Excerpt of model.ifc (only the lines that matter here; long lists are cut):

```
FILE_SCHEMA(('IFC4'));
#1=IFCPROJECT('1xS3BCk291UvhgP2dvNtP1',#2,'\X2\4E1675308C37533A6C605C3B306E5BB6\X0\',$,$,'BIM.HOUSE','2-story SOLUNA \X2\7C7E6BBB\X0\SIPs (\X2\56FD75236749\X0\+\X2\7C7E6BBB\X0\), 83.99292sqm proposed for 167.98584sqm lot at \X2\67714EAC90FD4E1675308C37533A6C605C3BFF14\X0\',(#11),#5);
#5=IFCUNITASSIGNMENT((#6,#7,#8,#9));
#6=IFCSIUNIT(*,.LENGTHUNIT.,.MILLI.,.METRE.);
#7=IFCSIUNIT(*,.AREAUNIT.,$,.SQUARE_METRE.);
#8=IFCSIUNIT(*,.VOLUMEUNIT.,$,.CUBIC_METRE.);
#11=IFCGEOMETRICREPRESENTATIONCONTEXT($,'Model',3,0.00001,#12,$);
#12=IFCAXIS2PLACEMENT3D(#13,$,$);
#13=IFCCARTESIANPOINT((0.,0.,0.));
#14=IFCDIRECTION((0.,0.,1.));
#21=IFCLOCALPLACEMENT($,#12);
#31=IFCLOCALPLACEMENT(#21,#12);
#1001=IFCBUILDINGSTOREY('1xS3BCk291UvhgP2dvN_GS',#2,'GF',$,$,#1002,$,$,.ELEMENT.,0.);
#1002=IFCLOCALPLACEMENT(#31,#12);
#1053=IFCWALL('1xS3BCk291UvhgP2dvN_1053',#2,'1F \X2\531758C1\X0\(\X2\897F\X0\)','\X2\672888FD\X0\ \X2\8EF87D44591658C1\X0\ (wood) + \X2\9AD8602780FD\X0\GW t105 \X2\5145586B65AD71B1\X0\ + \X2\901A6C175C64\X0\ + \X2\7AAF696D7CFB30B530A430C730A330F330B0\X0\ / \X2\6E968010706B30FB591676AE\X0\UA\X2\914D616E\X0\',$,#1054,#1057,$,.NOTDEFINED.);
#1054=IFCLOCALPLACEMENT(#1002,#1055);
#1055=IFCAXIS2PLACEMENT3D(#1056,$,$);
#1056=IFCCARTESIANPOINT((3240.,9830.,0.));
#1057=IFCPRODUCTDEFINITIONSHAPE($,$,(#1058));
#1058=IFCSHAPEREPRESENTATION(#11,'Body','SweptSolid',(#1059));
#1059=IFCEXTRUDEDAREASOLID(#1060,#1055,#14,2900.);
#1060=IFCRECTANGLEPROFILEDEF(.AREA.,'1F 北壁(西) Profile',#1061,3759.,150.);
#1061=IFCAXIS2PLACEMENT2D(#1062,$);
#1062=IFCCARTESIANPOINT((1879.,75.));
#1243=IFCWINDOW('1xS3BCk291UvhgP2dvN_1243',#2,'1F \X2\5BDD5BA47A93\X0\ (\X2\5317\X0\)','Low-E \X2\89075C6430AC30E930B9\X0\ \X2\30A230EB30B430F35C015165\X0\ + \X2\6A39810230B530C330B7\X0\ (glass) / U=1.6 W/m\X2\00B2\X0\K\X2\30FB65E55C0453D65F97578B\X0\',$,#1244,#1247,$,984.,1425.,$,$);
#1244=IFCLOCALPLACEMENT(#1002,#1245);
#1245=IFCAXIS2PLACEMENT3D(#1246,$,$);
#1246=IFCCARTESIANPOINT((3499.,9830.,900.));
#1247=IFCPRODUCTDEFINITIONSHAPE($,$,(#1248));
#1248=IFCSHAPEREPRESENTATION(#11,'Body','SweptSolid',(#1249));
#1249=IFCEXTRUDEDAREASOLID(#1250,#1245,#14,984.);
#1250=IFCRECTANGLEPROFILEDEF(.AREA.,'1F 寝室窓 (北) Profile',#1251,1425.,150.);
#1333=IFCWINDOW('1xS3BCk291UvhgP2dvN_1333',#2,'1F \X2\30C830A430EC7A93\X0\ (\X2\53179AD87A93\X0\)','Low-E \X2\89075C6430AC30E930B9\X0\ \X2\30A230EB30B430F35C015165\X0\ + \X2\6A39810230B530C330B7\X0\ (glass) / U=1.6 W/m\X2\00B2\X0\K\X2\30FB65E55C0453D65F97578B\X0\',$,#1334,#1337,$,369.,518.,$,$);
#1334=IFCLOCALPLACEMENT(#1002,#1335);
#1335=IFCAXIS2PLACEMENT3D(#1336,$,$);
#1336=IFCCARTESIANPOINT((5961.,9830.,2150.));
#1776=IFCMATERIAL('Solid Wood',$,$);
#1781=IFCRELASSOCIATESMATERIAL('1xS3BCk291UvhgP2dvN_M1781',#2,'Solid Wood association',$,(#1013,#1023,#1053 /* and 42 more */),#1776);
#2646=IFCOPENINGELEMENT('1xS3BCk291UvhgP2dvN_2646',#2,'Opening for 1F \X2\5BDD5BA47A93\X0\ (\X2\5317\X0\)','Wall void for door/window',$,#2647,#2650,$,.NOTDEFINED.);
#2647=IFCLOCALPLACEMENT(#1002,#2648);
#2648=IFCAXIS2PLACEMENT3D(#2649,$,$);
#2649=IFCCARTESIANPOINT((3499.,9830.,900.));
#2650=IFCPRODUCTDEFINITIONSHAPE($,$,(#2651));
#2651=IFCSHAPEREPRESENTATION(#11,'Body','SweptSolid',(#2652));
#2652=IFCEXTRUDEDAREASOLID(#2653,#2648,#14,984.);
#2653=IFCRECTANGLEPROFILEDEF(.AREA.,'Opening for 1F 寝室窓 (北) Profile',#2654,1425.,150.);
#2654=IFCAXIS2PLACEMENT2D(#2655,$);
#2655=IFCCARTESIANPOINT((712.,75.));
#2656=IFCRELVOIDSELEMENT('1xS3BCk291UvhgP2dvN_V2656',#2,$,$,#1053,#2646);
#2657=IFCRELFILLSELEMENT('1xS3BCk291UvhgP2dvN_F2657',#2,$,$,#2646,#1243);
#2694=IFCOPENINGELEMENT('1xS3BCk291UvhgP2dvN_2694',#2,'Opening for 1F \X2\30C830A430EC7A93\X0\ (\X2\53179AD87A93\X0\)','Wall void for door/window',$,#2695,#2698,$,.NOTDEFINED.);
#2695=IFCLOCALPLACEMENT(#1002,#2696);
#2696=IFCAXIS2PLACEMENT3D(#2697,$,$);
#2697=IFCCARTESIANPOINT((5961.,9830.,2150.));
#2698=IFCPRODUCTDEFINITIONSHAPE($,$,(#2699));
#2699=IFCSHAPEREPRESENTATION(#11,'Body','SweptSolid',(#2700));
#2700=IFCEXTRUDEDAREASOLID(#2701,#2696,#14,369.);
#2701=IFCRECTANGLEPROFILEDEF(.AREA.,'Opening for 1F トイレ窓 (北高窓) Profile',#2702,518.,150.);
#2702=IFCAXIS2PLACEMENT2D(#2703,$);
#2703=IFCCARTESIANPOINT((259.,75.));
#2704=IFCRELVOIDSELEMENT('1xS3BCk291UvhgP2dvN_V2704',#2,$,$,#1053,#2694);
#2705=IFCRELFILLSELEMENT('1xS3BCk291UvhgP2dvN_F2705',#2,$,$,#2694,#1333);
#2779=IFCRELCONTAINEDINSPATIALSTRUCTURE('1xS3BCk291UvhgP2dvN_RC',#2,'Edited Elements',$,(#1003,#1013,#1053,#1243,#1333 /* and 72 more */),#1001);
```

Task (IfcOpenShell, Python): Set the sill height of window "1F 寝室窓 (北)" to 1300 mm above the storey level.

```python
import numpy as np
import ifcopenshell
import ifcopenshell.api.geometry
import ifcopenshell.geom
import ifcopenshell.util.element
import ifcopenshell.util.placement
import ifcopenshell.util.shape
import ifcopenshell.util.unit

model = ifcopenshell.open("model.ifc")
unit_scale = ifcopenshell.util.unit.calculate_unit_scale(model)

window = model.by_guid("1xS3BCk291UvhgP2dvN_1243")
opening = window.FillsVoids[0].RelatingOpeningElement
storey = ifcopenshell.util.element.get_container(window, ifc_class="IfcBuildingStorey")
level = ifcopenshell.util.placement.get_local_placement(storey.ObjectPlacement)[2, 3]

# The opening's origin need not be at the sill, so measure its lowest point.
shape = ifcopenshell.geom.create_shape(ifcopenshell.geom.settings(), opening)
bottom = ifcopenshell.util.shape.get_shape_bottom_elevation(shape, shape.geometry) / unit_scale
dz = level + 1.3 / unit_scale - bottom

shift = np.array([0.0, 0.0, dz])
# The window is not placed relative to its opening, so move both.
for product in (opening, window):
    matrix = ifcopenshell.util.placement.get_local_placement(product.ObjectPlacement)
    matrix[:3, 3] += shift
    ifcopenshell.api.geometry.edit_object_placement(model, product=product, matrix=matrix, is_si=False)

print(f"moved by {dz * unit_scale:+.3f} m")

model.write("model-out.ifc")
```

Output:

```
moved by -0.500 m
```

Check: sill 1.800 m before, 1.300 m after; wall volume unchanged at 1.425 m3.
